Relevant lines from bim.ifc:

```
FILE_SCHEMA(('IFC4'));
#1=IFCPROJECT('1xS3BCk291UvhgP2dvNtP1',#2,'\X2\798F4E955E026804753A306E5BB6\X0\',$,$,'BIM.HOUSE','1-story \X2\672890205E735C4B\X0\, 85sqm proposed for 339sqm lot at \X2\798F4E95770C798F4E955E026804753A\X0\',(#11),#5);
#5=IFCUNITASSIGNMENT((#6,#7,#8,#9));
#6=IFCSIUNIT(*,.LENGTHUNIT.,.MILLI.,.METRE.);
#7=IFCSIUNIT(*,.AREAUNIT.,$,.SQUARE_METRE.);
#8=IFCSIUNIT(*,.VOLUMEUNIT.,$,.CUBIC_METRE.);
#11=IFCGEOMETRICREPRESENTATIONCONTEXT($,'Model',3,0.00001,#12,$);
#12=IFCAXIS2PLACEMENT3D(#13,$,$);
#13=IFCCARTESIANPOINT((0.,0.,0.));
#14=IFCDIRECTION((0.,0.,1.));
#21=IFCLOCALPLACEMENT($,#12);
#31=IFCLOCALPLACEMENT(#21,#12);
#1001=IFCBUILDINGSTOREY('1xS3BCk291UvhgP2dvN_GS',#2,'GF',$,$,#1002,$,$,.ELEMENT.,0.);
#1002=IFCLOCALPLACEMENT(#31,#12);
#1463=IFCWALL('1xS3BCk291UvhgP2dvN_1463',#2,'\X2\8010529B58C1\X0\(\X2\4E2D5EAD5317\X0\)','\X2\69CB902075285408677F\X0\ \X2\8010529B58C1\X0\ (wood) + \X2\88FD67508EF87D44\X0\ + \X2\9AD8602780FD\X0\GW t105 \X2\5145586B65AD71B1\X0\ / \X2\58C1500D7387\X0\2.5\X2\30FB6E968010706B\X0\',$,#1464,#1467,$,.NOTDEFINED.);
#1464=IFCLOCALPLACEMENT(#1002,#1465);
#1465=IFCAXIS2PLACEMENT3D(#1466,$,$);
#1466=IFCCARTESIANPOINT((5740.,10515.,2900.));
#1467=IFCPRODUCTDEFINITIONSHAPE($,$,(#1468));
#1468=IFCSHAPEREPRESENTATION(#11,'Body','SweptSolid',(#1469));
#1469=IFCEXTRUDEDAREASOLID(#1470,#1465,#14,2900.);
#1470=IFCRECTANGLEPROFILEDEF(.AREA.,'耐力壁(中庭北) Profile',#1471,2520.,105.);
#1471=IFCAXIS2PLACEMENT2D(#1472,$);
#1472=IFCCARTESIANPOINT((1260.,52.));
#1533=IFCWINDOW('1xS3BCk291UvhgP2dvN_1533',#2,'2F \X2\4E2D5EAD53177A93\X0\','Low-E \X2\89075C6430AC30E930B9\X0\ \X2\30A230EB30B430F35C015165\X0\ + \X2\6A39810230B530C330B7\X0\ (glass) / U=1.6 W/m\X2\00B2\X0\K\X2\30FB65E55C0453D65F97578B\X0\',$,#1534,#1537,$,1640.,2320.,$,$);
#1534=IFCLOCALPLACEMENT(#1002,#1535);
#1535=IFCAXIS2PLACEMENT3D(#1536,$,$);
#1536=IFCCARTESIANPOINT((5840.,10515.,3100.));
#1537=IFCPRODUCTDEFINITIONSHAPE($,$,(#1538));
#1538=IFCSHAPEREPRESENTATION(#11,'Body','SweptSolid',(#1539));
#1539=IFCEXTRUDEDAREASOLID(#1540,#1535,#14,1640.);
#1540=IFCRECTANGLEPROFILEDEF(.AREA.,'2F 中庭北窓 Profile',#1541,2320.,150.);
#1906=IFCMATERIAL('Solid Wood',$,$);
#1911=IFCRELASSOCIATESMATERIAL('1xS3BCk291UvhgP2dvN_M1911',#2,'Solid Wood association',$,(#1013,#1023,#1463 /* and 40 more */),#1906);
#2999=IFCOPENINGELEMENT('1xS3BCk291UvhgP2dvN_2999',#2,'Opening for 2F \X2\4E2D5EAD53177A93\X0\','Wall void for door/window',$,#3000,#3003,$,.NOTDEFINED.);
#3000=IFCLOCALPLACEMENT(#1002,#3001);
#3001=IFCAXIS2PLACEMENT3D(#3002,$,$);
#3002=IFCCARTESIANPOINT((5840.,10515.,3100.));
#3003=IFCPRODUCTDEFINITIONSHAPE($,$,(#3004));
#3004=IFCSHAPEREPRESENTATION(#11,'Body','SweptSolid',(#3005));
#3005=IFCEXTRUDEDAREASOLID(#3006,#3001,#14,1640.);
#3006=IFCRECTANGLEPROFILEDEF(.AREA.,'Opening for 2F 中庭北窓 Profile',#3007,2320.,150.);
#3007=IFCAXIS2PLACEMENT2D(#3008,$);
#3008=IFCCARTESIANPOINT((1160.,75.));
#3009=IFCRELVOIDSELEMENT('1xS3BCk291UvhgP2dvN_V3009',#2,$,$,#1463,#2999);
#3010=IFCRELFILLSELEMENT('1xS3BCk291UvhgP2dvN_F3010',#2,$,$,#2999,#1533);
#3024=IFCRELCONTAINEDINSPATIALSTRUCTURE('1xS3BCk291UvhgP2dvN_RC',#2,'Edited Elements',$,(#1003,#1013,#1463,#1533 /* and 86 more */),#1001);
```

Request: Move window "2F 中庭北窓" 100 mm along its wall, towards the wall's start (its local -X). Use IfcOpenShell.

```python
import ifcopenshell
import ifcopenshell.api.geometry
import ifcopenshell.util.placement
import ifcopenshell.util.unit

model = ifcopenshell.open("bim.ifc")
unit_scale = ifcopenshell.util.unit.calculate_unit_scale(model)

window = model.by_id(1533)
opening = window.FillsVoids[0].RelatingOpeningElement
wall = opening.VoidsElements[0].RelatingBuildingElement

wall_matrix = ifcopenshell.util.placement.get_local_placement(wall.ObjectPlacement)
shift = wall_matrix[:3, 0] * -0.1 / unit_scale
before = ifcopenshell.util.placement.get_local_placement(window.ObjectPlacement)[:3, 3].copy()

# The window is not placed relative to its opening, so move both.
for product in (opening, window):
    matrix = ifcopenshell.util.placement.get_local_placement(product.ObjectPlacement)
    matrix[:3, 3] += shift
    ifcopenshell.api.geometry.edit_object_placement(model, product=product, matrix=matrix, is_si=False)

after = ifcopenshell.util.placement.get_local_placement(window.ObjectPlacement)[:3, 3]
print("window moved by", (after - before).round(3) + 0.0)

model.write("bim_edited.ifc")
```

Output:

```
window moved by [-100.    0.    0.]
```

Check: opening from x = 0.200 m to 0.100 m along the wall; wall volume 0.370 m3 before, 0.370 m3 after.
